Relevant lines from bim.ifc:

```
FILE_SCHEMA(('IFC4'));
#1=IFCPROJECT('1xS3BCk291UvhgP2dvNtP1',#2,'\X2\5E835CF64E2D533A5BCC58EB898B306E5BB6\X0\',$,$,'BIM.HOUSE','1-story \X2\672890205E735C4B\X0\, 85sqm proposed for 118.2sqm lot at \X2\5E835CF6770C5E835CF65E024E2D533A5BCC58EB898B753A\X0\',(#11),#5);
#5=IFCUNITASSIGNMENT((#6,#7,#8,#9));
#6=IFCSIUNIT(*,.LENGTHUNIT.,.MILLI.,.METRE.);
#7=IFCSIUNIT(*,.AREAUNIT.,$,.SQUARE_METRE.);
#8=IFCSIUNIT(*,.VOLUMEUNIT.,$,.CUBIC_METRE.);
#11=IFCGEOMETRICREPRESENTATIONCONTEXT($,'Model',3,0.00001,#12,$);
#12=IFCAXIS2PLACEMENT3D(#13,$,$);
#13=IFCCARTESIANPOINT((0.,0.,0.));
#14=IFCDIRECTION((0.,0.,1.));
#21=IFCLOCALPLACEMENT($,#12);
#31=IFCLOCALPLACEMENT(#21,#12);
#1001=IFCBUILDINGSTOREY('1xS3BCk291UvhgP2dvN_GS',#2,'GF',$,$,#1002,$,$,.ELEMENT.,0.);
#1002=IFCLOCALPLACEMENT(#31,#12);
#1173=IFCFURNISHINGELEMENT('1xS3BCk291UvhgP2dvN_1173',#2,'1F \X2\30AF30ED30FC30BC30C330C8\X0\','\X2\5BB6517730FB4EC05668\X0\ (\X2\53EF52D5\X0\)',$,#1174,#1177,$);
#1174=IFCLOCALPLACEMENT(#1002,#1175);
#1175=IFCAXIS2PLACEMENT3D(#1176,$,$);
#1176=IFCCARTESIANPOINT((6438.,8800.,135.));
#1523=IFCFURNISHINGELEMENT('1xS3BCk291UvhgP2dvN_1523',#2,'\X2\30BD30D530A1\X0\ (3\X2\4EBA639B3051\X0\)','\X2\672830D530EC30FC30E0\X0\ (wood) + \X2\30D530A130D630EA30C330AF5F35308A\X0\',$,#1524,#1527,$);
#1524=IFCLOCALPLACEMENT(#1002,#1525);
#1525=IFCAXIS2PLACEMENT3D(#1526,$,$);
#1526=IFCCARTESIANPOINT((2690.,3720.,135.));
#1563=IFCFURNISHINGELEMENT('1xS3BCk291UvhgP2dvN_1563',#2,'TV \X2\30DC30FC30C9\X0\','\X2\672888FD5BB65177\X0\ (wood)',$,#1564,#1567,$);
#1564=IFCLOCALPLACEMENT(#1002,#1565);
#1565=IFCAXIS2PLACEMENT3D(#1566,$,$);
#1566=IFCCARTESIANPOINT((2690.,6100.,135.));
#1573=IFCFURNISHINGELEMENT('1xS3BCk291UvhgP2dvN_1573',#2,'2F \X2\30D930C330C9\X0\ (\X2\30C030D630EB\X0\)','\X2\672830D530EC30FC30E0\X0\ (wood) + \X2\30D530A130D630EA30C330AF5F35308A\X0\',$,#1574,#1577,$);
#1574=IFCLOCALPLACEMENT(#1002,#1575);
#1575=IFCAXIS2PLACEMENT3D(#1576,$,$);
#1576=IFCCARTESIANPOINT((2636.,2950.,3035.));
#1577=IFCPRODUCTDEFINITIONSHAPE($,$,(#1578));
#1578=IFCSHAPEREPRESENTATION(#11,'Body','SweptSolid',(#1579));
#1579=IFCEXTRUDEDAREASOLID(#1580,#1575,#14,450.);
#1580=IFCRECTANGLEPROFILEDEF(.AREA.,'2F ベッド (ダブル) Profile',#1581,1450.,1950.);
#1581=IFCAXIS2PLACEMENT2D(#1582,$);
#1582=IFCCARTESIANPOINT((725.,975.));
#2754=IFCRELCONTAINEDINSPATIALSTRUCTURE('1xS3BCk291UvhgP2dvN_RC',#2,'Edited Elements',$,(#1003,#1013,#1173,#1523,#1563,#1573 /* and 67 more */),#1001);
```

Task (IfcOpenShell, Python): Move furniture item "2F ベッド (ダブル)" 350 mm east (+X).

```python
import ifcopenshell
import ifcopenshell.api.geometry
import ifcopenshell.util.placement

model = ifcopenshell.open("bim.ifc")

item = model.by_guid("1xS3BCk291UvhgP2dvN_1573")
matrix = ifcopenshell.util.placement.get_local_placement(item.ObjectPlacement)
matrix[0, 3] += 350.0
ifcopenshell.api.geometry.edit_object_placement(model, product=item, matrix=matrix, is_si=False)

print(ifcopenshell.util.placement.get_local_placement(item.ObjectPlacement).round(3) + 0.0)

model.write("bim_updated.ifc")
```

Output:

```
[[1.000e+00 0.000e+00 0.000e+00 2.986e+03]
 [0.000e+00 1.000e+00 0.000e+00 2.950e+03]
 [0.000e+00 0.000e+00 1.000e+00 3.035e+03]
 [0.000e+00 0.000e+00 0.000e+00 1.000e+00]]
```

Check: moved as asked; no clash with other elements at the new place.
